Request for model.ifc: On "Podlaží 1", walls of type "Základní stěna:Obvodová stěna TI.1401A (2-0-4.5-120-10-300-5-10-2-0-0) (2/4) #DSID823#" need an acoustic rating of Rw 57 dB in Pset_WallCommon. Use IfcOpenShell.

First a look at what the model holds.

```python
import ifcopenshell
import ifcopenshell.util.element

model = ifcopenshell.open("model.ifc")
print(model.schema)
storey = next(s for s in model.by_type("IfcBuildingStorey") if s.Name == "Podlaží 1")
walls = [e for e in ifcopenshell.util.element.get_decomposition(storey) if e.is_a("IfcWall")]
seen = {}
for e in walls:
    element_type = ifcopenshell.util.element.get_type(e)
    key = (element_type.Name if element_type != e and element_type else None, ifcopenshell.util.element.get_pset(e, "Pset_WallCommon", "AcousticRating"))
    seen[key] = seen.get(key, 0) + 1
for (name, value), count in sorted(seen.items(), key=str):
    print(count, "x", name, "|", value)
```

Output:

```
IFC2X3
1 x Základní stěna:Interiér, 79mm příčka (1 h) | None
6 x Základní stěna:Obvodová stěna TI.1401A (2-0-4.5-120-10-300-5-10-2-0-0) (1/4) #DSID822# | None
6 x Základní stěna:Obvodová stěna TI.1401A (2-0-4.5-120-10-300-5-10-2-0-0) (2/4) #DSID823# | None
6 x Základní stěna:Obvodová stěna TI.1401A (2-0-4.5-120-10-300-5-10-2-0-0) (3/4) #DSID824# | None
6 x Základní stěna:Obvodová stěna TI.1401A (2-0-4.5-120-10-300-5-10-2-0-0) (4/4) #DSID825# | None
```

```python
import ifcopenshell
import ifcopenshell.api.pset
import ifcopenshell.util.element

model = ifcopenshell.open("model.ifc")

storey = next(s for s in model.by_type("IfcBuildingStorey") if s.Name == "Podlaží 1")
walls = [e for e in ifcopenshell.util.element.get_decomposition(storey) if e.is_a("IfcWall")]

count = 0
for e in walls:
    element_type = ifcopenshell.util.element.get_type(e)
    if element_type in (None, e) or element_type.Name != "Základní stěna:Obvodová stěna TI.1401A (2-0-4.5-120-10-300-5-10-2-0-0) (2/4) #DSID823#":
        continue
    # add_pset returns the element's existing set when there is one.
    pset = ifcopenshell.api.pset.add_pset(model, product=e, name="Pset_WallCommon")
    ifcopenshell.api.pset.edit_pset(model, pset=pset, properties={"AcousticRating": "Rw 57 dB"})
    count += 1

print(count, "walls updated")

model.write("model_edited.ifc")
```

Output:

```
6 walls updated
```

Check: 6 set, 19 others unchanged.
